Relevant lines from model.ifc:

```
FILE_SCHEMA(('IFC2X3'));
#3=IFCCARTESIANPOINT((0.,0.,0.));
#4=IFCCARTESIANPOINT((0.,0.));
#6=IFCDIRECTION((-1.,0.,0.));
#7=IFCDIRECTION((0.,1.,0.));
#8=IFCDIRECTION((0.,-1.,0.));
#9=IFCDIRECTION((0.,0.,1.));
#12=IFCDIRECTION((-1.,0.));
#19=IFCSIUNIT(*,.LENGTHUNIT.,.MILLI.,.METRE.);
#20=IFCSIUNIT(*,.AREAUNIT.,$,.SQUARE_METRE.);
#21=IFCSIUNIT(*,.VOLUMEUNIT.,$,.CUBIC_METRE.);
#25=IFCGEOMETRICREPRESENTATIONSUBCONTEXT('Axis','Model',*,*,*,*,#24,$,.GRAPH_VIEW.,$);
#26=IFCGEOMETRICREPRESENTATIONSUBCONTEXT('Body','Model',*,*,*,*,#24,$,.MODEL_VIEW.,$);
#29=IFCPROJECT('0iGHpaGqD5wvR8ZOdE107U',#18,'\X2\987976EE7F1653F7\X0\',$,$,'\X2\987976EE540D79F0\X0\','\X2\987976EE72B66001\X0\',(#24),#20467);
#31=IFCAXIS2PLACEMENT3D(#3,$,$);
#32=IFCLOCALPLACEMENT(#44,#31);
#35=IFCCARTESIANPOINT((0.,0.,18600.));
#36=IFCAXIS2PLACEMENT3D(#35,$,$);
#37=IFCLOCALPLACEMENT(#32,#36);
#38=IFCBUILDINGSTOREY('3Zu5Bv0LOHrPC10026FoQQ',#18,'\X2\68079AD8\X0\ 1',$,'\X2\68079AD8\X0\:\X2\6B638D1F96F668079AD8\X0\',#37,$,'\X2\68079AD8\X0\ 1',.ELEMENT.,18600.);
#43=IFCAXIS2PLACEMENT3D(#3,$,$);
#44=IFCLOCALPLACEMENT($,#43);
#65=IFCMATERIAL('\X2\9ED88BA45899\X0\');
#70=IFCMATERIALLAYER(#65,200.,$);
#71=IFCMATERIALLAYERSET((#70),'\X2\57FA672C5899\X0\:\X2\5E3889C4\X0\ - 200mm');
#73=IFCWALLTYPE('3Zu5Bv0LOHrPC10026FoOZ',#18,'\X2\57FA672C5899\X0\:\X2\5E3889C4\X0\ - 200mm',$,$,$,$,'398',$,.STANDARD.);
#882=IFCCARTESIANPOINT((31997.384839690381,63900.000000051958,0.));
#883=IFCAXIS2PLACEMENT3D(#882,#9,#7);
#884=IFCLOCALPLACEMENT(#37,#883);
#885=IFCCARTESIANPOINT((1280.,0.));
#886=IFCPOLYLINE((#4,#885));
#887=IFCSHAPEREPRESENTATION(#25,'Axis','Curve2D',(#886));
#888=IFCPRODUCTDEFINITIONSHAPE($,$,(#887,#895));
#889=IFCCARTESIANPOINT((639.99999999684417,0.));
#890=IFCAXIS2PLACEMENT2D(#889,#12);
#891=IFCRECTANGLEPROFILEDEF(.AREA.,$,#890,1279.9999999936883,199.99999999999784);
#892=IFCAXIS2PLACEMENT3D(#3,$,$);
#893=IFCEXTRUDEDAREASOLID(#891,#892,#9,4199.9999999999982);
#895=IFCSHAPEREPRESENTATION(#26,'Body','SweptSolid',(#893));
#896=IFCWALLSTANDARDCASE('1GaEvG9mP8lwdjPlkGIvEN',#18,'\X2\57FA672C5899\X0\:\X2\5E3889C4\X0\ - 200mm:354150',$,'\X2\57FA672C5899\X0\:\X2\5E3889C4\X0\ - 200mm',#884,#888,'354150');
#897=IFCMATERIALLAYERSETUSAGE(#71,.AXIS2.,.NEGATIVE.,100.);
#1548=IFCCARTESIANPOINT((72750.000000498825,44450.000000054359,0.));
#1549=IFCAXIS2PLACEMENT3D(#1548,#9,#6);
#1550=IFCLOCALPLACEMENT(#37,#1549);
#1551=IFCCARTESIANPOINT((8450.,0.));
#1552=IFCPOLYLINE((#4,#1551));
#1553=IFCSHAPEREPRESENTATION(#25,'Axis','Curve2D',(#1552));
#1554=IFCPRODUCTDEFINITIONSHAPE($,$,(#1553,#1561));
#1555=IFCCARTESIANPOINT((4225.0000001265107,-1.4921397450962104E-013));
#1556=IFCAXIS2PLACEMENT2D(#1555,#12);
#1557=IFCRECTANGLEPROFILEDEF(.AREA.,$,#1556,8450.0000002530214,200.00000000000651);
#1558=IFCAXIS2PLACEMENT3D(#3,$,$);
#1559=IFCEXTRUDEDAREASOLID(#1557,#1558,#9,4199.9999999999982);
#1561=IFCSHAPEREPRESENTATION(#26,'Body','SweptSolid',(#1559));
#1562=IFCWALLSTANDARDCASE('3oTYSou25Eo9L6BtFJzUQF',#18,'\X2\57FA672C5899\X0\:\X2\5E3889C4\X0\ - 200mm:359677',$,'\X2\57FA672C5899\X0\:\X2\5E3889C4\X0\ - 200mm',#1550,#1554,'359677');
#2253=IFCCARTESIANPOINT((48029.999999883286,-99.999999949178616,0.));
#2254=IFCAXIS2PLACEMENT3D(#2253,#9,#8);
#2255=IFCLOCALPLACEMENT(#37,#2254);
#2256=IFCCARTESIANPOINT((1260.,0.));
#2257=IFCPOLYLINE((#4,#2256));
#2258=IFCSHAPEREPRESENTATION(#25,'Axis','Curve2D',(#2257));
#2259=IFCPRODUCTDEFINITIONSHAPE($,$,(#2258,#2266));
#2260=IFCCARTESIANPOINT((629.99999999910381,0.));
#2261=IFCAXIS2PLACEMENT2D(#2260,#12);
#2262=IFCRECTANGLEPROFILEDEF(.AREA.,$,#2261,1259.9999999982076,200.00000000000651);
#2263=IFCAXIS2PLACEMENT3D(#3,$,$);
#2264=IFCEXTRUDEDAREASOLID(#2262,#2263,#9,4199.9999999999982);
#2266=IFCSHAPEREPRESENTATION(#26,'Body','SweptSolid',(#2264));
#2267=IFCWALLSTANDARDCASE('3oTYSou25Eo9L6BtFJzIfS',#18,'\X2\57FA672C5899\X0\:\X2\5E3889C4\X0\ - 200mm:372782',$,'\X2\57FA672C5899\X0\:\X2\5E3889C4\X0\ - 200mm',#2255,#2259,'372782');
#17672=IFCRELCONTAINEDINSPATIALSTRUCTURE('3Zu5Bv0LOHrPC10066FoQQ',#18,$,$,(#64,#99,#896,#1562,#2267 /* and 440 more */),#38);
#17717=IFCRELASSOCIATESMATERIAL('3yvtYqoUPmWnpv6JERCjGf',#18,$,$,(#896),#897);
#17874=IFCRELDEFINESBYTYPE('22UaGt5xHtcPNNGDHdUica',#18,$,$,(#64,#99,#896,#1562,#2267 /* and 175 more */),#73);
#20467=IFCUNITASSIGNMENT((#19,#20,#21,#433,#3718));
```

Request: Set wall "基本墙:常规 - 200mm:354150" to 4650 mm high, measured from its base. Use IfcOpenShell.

```python
import ifcopenshell
import ifcopenshell.geom
import ifcopenshell.util.representation
import ifcopenshell.util.shape
import ifcopenshell.util.unit

model = ifcopenshell.open("model.ifc")
unit_scale = ifcopenshell.util.unit.calculate_unit_scale(model)
settings = ifcopenshell.geom.settings()


def volume(element):
    """Net volume in cubic metres, openings subtracted."""
    shape = ifcopenshell.geom.create_shape(settings, element)
    return ifcopenshell.util.shape.get_volume(shape.geometry)


wall = model.by_guid("1GaEvG9mP8lwdjPlkGIvEN")
before = volume(wall)

body = ifcopenshell.util.representation.get_representation(wall, "Model", "Body")
solid = body.Items[0]
old_height = solid.Depth
solid.Depth = 4.65 / unit_scale
after = volume(wall)

print(f"height {old_height:g} -> {solid.Depth:g}, volume {before:.3f} -> {after:.3f} m3")

model.write("model_updated.ifc")
```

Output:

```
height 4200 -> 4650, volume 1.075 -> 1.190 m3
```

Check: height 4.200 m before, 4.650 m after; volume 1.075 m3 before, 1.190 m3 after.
